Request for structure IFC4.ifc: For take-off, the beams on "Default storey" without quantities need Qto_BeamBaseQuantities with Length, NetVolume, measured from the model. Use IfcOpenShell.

First a look at what the model holds.

```python
import ifcopenshell
import ifcopenshell.util.element
import ifcopenshell.util.unit

model = ifcopenshell.open("structure IFC4.ifc")
print(model.schema)
for unit_type in ("LENGTHUNIT", "AREAUNIT", "VOLUMEUNIT"):
    print(unit_type, ifcopenshell.util.unit.calculate_unit_scale(model, unit_type))
storey = next(s for s in model.by_type("IfcBuildingStorey") if s.Name == "Default storey")
beams = [e for e in ifcopenshell.util.element.get_decomposition(storey) if e.is_a("IfcBeam")]
for e in sorted(beams, key=lambda e: e.id()):
    print(e.id(), e.is_a(), e.Name, list(ifcopenshell.util.element.get_psets(e, qtos_only=True)), sep=" | ")
```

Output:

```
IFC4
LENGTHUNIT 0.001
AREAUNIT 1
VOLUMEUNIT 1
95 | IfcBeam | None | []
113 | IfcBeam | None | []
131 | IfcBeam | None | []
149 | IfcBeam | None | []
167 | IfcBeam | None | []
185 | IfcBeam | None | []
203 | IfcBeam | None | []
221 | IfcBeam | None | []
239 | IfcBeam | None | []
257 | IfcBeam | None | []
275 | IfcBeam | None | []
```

```python
import ifcopenshell
import ifcopenshell.api.pset
import ifcopenshell.geom
import ifcopenshell.util.element
import ifcopenshell.util.shape
import ifcopenshell.util.unit

model = ifcopenshell.open("structure IFC4.ifc")
unit_scale = ifcopenshell.util.unit.calculate_unit_scale(model)
volume_scale = ifcopenshell.util.unit.calculate_unit_scale(model, "VOLUMEUNIT")
settings = ifcopenshell.geom.settings()

storey = next(s for s in model.by_type("IfcBuildingStorey") if s.Name == "Default storey")
beams = [e for e in ifcopenshell.util.element.get_decomposition(storey) if e.is_a("IfcBeam")]

for e in sorted(beams, key=lambda e: e.id()):
    if ifcopenshell.util.element.get_psets(e, qtos_only=True, should_inherit=False):
        continue
    # Geometry comes back in metres, in the element's own axes.
    shape = ifcopenshell.geom.create_shape(settings, e)
    values = {
        "Length": ifcopenshell.util.shape.get_max_xyz(shape.geometry) / unit_scale,
        "NetVolume": ifcopenshell.util.shape.get_volume(shape.geometry) / volume_scale,
    }
    qto = ifcopenshell.api.pset.add_qto(model, product=e, name="Qto_BeamBaseQuantities")
    ifcopenshell.api.pset.edit_qto(model, qto=qto, properties=values)
    print(e.id(), {k: round(v, 3) for k, v in values.items()})

model.write("structure IFC4_v2.ifc")
```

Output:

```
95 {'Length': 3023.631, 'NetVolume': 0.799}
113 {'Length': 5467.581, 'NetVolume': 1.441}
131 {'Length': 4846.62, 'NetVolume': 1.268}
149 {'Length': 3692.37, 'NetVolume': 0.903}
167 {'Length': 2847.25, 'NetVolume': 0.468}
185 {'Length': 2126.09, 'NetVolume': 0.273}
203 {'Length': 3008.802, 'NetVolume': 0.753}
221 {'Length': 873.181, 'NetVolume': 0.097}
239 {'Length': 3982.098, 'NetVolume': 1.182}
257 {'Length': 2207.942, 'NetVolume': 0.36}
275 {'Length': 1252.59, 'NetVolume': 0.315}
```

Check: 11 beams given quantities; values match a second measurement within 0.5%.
